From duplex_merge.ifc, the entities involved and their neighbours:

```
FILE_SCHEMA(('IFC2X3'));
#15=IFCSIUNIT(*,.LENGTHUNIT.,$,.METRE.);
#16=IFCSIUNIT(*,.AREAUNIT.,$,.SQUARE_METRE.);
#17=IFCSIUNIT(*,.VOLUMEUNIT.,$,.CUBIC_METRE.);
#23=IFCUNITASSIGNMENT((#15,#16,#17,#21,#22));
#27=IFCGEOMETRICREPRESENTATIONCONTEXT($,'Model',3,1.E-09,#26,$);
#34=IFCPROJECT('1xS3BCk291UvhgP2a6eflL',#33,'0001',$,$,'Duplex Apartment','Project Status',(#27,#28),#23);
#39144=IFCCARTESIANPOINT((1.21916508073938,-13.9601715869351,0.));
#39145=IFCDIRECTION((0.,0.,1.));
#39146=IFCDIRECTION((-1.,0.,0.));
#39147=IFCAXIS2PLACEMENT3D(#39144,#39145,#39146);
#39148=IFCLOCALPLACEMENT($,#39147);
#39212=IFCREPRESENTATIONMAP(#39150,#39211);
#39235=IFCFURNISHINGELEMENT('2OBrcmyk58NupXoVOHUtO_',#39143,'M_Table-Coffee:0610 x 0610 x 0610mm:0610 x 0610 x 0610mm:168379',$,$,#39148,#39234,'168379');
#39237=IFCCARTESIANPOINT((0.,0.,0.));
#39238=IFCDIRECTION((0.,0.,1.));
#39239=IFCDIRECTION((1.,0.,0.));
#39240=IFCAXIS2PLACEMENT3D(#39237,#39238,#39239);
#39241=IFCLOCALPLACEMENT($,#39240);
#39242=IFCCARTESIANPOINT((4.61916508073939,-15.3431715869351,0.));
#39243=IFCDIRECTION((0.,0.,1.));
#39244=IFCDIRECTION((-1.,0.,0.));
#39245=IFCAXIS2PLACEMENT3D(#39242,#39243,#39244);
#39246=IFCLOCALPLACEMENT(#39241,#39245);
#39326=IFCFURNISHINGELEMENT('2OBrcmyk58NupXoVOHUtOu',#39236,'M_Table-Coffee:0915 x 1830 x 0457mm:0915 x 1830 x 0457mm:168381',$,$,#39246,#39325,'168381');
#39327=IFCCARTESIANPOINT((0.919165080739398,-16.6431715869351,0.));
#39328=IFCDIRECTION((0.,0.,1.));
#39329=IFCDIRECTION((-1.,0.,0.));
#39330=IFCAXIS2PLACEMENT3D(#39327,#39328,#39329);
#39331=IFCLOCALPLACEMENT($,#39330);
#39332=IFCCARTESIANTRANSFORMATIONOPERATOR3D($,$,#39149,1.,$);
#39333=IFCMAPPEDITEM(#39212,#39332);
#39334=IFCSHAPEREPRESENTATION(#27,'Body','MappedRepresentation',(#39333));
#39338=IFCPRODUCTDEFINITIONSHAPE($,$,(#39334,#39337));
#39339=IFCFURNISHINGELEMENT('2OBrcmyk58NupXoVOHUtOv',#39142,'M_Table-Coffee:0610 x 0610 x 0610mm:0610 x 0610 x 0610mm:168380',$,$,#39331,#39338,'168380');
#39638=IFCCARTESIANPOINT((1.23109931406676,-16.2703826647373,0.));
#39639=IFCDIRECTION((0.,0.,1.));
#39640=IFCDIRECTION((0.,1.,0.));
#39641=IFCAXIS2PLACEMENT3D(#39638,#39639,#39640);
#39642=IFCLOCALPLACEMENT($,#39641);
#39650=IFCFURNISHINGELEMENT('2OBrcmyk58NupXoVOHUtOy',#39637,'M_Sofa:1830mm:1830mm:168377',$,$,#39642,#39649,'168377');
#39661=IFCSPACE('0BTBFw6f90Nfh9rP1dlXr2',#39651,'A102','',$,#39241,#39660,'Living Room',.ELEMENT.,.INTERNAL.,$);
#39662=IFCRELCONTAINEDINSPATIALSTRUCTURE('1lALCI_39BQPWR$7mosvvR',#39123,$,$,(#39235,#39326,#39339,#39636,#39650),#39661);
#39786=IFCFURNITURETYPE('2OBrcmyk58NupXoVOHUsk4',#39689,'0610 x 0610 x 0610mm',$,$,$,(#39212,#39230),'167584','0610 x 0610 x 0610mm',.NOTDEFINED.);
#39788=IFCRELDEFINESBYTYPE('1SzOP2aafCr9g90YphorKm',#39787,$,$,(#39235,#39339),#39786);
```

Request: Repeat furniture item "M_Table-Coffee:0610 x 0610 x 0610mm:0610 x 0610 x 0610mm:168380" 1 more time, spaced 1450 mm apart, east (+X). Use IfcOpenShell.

```python
import numpy as np
import ifcopenshell
import ifcopenshell.api.geometry
import ifcopenshell.api.root
import ifcopenshell.util.element
import ifcopenshell.util.placement
import ifcopenshell.util.unit

model = ifcopenshell.open("duplex_merge.ifc")
unit_scale = ifcopenshell.util.unit.calculate_unit_scale(model)


def reuse_history(source, copy):
    """copy_class also copies each property set's owner history, people and application; keep the originals."""
    for rel in copy.IsDefinedBy:
        if rel.is_a("IfcRelDefinesByProperties") and (history := rel.RelatingPropertyDefinition.OwnerHistory):
            rel.RelatingPropertyDefinition.OwnerHistory = source.OwnerHistory
            ifcopenshell.util.element.remove_deep2(model, history)


source = model.by_guid("2OBrcmyk58NupXoVOHUtOv")
base = ifcopenshell.util.placement.get_local_placement(source.ObjectPlacement)
step = np.array([1.0, 0.0, 0.0]) * 1.45 / unit_scale

for i in range(1, 2):
    copy = ifcopenshell.api.root.copy_class(model, product=source)
    copy.Representation = ifcopenshell.util.element.copy_deep(
        model, source.Representation, exclude=["IfcGeometricRepresentationContext", "IfcRepresentationMap"]
    )
    copy.Name = "M_Table-Coffee:0610 x 0610 x 0610mm:0610 x 0610 x 0610mm"
    copy.Tag = None
    reuse_history(source, copy)
    matrix = base.copy()
    matrix[:3, 3] += i * step
    print("added at", matrix[:3, 3].round(3) + 0.0)
    ifcopenshell.api.geometry.edit_object_placement(model, product=copy, matrix=matrix, is_si=False)

model.write("duplex_merge_updated.ifc")
```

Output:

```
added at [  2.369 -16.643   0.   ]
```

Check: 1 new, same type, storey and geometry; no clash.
